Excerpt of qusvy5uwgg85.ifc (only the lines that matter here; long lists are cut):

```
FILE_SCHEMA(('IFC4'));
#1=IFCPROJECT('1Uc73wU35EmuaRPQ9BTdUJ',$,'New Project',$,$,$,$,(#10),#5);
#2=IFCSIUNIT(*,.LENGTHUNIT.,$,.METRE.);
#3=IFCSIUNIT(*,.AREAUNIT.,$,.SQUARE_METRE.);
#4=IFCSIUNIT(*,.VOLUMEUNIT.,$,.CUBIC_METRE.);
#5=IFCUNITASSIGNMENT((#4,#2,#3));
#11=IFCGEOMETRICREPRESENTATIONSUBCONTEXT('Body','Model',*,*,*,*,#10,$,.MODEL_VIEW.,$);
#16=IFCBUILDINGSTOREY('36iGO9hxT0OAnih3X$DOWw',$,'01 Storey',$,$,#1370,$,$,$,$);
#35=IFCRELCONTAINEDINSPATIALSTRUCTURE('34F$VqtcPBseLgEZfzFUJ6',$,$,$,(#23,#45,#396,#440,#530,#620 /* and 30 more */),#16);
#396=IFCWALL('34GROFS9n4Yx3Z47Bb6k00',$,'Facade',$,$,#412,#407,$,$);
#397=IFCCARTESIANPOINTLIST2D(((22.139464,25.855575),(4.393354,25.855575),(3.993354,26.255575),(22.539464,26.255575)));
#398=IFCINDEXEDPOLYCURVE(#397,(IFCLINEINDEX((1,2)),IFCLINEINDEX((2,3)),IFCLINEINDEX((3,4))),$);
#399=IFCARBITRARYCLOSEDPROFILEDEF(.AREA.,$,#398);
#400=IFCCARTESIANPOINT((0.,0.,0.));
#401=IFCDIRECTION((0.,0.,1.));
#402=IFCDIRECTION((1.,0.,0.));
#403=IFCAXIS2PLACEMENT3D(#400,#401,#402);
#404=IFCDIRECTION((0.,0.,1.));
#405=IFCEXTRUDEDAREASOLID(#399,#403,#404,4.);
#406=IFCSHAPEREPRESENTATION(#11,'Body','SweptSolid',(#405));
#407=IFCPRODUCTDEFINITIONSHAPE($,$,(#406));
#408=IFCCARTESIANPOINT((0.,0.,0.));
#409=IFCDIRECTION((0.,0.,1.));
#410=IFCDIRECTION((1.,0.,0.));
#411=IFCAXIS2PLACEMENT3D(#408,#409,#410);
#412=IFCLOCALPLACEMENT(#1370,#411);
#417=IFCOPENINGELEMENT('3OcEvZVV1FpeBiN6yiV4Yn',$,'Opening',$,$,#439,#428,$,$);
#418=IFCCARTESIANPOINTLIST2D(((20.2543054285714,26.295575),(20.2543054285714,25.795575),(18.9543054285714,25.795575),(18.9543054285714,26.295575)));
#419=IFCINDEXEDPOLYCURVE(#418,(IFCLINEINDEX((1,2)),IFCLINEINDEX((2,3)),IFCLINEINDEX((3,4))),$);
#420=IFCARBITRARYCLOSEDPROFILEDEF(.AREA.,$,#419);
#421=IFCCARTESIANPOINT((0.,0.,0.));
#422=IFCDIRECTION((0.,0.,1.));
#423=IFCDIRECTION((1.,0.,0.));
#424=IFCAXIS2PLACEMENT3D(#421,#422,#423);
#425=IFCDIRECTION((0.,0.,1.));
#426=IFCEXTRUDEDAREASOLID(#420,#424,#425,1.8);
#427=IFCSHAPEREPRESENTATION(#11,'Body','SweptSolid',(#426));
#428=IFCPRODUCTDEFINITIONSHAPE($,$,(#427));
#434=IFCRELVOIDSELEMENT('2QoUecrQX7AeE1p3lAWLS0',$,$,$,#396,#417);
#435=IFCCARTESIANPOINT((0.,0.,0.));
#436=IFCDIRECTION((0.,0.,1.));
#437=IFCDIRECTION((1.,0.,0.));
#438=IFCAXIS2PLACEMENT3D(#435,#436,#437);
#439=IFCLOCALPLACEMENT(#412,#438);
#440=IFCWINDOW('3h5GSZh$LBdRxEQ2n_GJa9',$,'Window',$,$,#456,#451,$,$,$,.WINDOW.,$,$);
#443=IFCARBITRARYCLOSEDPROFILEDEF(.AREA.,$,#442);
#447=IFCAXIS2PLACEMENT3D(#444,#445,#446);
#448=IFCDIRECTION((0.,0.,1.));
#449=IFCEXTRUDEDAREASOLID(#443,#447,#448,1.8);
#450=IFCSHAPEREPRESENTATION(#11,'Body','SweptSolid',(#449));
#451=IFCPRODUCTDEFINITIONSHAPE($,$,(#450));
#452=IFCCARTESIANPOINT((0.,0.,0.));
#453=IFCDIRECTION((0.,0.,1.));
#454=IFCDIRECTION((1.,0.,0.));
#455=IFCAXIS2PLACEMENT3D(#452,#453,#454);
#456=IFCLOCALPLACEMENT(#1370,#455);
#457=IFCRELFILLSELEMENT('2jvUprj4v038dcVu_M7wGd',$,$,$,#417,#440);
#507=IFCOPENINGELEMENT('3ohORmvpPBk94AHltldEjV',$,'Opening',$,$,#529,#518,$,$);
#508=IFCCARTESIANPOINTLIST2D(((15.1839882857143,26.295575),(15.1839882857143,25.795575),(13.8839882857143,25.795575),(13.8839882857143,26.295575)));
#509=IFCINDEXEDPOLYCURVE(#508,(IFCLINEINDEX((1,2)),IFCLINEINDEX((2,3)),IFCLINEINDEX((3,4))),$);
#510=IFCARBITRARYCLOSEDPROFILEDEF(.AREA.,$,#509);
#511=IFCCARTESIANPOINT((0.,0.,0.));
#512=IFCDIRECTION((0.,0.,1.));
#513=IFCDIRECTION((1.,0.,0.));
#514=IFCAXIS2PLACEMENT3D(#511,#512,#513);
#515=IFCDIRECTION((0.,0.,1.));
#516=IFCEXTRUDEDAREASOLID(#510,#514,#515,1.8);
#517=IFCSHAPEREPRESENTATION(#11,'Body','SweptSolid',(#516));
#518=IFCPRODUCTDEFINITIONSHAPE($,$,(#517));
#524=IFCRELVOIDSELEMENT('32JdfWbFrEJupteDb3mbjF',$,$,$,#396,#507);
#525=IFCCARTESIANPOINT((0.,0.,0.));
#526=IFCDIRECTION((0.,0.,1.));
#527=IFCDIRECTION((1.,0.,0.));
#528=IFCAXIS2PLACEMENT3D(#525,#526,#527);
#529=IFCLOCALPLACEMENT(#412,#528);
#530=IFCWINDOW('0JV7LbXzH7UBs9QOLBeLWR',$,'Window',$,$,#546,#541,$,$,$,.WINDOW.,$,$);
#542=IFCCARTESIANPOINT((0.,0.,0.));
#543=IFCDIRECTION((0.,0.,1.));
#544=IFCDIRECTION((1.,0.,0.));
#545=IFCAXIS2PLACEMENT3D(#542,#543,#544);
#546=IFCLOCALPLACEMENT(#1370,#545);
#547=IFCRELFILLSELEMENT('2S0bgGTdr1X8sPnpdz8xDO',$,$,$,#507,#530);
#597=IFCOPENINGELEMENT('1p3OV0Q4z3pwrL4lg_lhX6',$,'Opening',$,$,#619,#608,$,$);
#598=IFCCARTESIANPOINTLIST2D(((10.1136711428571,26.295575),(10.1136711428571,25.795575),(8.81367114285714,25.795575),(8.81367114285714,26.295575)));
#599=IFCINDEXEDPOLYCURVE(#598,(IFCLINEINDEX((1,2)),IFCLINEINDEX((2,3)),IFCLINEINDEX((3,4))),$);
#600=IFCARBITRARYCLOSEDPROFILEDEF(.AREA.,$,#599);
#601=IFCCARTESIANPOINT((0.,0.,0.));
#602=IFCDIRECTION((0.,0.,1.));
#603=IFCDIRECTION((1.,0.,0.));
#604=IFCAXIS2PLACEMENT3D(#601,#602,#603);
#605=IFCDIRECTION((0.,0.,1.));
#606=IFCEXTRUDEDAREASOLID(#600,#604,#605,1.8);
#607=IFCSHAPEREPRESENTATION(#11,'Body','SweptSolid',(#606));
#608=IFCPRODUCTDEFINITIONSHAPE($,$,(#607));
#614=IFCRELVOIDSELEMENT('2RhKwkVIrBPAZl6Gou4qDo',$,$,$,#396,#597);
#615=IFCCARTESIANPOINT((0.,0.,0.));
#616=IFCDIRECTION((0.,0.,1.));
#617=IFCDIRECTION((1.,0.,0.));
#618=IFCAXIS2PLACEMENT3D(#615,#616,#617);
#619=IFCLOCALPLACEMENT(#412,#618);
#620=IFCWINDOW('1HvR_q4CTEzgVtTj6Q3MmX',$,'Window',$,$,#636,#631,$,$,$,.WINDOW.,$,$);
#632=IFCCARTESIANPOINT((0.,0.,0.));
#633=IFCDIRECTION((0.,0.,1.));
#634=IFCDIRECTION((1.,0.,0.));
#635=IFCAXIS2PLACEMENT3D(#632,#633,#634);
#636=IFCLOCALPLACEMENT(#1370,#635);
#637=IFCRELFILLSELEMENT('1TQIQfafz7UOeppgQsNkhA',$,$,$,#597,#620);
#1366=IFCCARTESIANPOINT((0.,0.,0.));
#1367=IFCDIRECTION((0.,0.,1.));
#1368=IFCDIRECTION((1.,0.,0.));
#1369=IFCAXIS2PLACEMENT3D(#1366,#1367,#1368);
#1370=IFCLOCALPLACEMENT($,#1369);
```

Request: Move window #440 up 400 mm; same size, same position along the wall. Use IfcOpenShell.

```python
import numpy as np
import ifcopenshell
import ifcopenshell.api.geometry
import ifcopenshell.util.placement
import ifcopenshell.util.unit

model = ifcopenshell.open("qusvy5uwgg85.ifc")
unit_scale = ifcopenshell.util.unit.calculate_unit_scale(model)

window = model.by_id(440)
opening = window.FillsVoids[0].RelatingOpeningElement
dz = 0.4

shift = np.array([0.0, 0.0, dz])
# The window is not placed relative to its opening, so move both.
for product in (opening, window):
    matrix = ifcopenshell.util.placement.get_local_placement(product.ObjectPlacement)
    matrix[:3, 3] += shift
    ifcopenshell.api.geometry.edit_object_placement(model, product=product, matrix=matrix, is_si=False)

print(f"moved by {dz * unit_scale:+.3f} m")

model.write("qusvy5uwgg85_updated.ifc")
```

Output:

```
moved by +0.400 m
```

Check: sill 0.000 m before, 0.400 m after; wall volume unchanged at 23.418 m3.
